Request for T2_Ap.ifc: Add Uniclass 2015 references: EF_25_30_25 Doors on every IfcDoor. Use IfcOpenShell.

First a look at what the model holds.

```python
import ifcopenshell

model = ifcopenshell.open("T2_Ap.ifc")
print(model.schema)
print("classifications:", [c.Name for c in model.by_type("IfcClassification")])
for ifc_class in ("IfcDoor", "IfcRoof", "IfcStair", "IfcWall", "IfcWindow"):
    print(ifc_class, len(model.by_type(ifc_class)))
```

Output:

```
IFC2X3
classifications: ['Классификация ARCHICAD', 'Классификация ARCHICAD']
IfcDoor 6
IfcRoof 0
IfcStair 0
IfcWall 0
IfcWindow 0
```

```python
import ifcopenshell
import ifcopenshell.api.classification

model = ifcopenshell.open("T2_Ap.ifc")

# IFC2X3 requires Source and Edition and has no link from the project to the system.
system = model.create_entity("IfcClassification", Source="NBS", Edition="2015", Name="Uniclass 2015")

codes = {
    "IfcDoor": ("EF_25_30_25", "Doors"),
}
for ifc_class, (code, name) in codes.items():
    products = model.by_type(ifc_class)
    ifcopenshell.api.classification.add_reference(
        model, products=products, classification=system, identification=code, name=name
    )
    print(code, len(products))

model.write("T2_Ap-out.ifc")
```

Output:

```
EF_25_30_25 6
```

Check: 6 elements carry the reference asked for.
